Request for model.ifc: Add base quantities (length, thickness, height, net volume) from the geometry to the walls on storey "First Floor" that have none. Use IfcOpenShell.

First a look at what the model holds.

```python
import ifcopenshell
import ifcopenshell.util.element
import ifcopenshell.util.unit

model = ifcopenshell.open("model.ifc")
print(model.schema)
for unit_type in ("LENGTHUNIT", "AREAUNIT", "VOLUMEUNIT"):
    print(unit_type, ifcopenshell.util.unit.calculate_unit_scale(model, unit_type))
storey = next(s for s in model.by_type("IfcBuildingStorey") if s.Name == "First Floor")
walls = [e for e in ifcopenshell.util.element.get_decomposition(storey) if e.is_a("IfcWall")]
for e in sorted(walls, key=lambda e: e.id()):
    print(e.id(), e.is_a(), e.Name, list(ifcopenshell.util.element.get_psets(e, qtos_only=True)), sep=" | ")
```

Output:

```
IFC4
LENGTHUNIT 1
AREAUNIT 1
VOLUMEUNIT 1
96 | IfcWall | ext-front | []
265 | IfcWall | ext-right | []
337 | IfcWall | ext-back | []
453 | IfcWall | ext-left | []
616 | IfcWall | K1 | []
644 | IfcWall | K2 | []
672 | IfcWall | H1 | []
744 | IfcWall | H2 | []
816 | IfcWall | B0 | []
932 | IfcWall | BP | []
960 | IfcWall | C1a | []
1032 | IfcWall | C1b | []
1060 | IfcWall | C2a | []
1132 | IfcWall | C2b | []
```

```python
import ifcopenshell
import ifcopenshell.api.pset
import ifcopenshell.geom
import ifcopenshell.util.element
import ifcopenshell.util.shape
import ifcopenshell.util.unit

model = ifcopenshell.open("model.ifc")
unit_scale = ifcopenshell.util.unit.calculate_unit_scale(model)
volume_scale = ifcopenshell.util.unit.calculate_unit_scale(model, "VOLUMEUNIT")
settings = ifcopenshell.geom.settings()

storey = next(s for s in model.by_type("IfcBuildingStorey") if s.Name == "First Floor")
walls = [e for e in ifcopenshell.util.element.get_decomposition(storey) if e.is_a("IfcWall")]

for e in sorted(walls, key=lambda e: e.id()):
    if ifcopenshell.util.element.get_psets(e, qtos_only=True, should_inherit=False):
        continue
    # Geometry comes back in metres, in the element's own axes.
    shape = ifcopenshell.geom.create_shape(settings, e)
    values = {
        "Length": ifcopenshell.util.shape.get_x(shape.geometry) / unit_scale,
        "Width": ifcopenshell.util.shape.get_y(shape.geometry) / unit_scale,
        "Height": ifcopenshell.util.shape.get_z(shape.geometry) / unit_scale,
        "NetVolume": ifcopenshell.util.shape.get_volume(shape.geometry) / volume_scale,
    }
    qto = ifcopenshell.api.pset.add_qto(model, product=e, name="Qto_WallBaseQuantities")
    ifcopenshell.api.pset.edit_qto(model, qto=qto, properties=values)
    print(e.id(), {k: round(v, 3) for k, v in values.items()})

model.write("model-out.ifc")
```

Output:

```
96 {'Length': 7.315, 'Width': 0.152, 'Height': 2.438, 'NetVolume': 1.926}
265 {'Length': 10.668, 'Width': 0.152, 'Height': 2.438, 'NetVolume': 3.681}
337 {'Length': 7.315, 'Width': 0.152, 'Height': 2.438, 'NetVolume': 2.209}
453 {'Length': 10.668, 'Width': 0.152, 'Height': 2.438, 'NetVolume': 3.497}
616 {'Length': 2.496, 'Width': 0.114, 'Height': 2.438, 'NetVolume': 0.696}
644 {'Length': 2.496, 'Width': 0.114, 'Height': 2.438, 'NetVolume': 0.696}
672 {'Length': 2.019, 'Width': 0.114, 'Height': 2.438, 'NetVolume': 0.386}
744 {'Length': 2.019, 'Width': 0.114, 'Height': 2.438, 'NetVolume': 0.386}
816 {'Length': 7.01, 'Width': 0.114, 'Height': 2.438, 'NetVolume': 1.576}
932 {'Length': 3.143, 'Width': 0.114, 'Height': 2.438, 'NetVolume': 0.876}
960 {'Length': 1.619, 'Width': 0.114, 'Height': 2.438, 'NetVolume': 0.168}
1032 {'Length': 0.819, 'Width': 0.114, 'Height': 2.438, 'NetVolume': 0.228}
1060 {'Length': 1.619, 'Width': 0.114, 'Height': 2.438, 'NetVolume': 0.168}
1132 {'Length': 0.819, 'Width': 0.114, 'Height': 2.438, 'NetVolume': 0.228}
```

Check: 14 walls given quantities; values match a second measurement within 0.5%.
